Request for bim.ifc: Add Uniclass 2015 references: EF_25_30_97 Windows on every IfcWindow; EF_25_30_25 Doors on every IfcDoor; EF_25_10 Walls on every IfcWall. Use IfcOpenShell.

First a look at what the model holds.

```python
import ifcopenshell

model = ifcopenshell.open("bim.ifc")
print(model.schema)
print("classifications:", [c.Name for c in model.by_type("IfcClassification")])
for ifc_class in ("IfcDoor", "IfcRoof", "IfcStair", "IfcWall", "IfcWindow"):
    print(ifc_class, len(model.by_type(ifc_class)))
```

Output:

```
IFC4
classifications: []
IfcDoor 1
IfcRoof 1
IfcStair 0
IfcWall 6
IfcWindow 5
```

```python
import ifcopenshell
import ifcopenshell.api.classification

model = ifcopenshell.open("bim.ifc")

system = ifcopenshell.api.classification.add_classification(model, classification="Uniclass 2015")

codes = {
    "IfcWindow": ("EF_25_30_97", "Windows"),
    "IfcDoor": ("EF_25_30_25", "Doors"),
    "IfcWall": ("EF_25_10", "Walls"),
}
for ifc_class, (code, name) in codes.items():
    products = model.by_type(ifc_class)
    ifcopenshell.api.classification.add_reference(
        model, products=products, classification=system, identification=code, name=name
    )
    print(code, len(products))

model.write("bim_rev.ifc")
```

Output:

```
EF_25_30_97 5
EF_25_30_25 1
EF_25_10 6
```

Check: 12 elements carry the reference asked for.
